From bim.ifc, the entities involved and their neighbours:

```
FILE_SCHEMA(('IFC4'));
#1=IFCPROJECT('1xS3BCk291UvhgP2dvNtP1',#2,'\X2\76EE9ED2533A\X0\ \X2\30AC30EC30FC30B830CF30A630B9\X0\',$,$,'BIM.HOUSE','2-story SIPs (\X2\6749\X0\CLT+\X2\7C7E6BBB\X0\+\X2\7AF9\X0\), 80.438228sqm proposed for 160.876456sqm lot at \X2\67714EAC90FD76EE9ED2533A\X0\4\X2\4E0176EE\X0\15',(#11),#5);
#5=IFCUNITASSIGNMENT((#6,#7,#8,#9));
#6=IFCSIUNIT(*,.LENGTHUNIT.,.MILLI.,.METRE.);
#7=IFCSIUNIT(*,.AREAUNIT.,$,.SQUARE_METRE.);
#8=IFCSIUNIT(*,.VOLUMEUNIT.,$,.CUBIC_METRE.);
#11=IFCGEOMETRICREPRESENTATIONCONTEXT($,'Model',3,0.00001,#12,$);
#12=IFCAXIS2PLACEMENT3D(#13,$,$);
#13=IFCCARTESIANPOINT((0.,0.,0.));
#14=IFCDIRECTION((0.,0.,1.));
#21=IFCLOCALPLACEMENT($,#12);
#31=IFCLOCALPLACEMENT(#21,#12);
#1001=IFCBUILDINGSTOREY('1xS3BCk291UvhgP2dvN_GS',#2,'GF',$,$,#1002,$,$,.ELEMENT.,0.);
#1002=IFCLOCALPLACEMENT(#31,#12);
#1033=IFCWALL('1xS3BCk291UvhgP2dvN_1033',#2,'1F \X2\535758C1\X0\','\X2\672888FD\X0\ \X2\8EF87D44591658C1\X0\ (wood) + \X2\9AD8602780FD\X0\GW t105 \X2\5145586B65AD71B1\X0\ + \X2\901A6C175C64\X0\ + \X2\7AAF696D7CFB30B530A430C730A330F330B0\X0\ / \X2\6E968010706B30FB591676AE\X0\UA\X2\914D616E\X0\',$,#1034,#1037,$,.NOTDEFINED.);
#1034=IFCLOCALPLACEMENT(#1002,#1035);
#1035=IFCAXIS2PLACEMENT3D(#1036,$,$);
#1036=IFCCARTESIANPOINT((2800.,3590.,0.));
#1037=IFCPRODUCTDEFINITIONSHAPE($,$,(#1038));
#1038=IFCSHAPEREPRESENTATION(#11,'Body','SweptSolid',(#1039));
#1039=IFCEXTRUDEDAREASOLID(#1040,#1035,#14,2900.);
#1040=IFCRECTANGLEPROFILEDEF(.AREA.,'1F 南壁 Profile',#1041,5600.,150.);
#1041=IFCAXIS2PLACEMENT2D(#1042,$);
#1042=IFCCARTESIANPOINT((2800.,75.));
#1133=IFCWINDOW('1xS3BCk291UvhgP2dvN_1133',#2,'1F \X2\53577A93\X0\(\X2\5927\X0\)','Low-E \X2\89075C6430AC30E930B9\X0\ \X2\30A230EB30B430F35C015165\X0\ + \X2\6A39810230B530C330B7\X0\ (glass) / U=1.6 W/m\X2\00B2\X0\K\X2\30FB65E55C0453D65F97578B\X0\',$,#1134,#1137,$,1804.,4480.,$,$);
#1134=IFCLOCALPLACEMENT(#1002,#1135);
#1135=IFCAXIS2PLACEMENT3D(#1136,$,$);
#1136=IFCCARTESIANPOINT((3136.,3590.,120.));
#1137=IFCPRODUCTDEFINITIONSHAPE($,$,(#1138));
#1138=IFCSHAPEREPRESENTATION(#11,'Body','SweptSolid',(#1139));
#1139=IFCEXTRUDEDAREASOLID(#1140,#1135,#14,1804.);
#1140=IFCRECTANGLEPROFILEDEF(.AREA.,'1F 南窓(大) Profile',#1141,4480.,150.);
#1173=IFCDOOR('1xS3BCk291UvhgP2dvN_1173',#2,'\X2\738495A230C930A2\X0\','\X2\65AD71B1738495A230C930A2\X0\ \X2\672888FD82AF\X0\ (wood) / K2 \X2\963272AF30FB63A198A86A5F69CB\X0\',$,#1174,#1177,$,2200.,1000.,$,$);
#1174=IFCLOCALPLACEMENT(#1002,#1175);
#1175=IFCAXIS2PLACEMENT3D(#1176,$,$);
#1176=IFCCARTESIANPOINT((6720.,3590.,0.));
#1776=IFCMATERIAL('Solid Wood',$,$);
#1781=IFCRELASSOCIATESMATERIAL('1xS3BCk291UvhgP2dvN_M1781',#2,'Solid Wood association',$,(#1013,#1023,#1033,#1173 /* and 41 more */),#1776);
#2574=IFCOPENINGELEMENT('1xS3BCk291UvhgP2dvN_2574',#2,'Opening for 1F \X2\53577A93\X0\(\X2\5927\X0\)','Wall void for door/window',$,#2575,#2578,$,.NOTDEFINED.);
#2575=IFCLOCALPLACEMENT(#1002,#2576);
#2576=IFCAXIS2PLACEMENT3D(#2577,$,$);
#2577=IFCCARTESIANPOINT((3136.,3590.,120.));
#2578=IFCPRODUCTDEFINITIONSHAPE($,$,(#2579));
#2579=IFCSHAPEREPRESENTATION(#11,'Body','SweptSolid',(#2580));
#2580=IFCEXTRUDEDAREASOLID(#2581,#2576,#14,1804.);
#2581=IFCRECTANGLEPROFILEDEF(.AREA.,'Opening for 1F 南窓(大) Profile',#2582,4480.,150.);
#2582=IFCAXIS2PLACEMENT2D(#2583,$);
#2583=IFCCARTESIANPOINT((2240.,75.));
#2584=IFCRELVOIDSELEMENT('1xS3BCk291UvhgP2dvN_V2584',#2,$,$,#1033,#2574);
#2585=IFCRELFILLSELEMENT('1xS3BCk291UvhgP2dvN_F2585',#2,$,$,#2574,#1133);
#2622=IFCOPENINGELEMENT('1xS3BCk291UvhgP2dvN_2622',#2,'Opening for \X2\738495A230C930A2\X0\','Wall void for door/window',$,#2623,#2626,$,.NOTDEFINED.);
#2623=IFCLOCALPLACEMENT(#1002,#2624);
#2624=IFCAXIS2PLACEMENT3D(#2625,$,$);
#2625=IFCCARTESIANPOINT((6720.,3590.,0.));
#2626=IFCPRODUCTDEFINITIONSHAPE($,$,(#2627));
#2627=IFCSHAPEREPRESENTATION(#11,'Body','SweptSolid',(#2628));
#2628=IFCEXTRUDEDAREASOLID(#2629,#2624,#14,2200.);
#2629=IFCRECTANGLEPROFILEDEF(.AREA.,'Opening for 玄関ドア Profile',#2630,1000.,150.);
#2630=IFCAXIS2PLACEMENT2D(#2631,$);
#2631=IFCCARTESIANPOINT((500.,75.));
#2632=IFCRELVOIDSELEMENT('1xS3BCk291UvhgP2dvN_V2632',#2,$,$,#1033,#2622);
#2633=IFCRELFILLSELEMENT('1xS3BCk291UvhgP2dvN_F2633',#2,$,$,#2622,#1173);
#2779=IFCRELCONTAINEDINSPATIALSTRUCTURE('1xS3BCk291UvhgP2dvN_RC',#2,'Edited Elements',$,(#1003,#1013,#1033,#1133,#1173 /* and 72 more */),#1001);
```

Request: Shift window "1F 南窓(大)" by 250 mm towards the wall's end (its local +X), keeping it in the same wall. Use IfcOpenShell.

```python
import ifcopenshell
import ifcopenshell.api.geometry
import ifcopenshell.util.placement

model = ifcopenshell.open("bim.ifc")

window = model.by_guid("1xS3BCk291UvhgP2dvN_1133")
opening = window.FillsVoids[0].RelatingOpeningElement
wall = opening.VoidsElements[0].RelatingBuildingElement

wall_matrix = ifcopenshell.util.placement.get_local_placement(wall.ObjectPlacement)
shift = wall_matrix[:3, 0] * 250.0
before = ifcopenshell.util.placement.get_local_placement(window.ObjectPlacement)[:3, 3].copy()

# The window is not placed relative to its opening, so move both.
for product in (opening, window):
    matrix = ifcopenshell.util.placement.get_local_placement(product.ObjectPlacement)
    matrix[:3, 3] += shift
    ifcopenshell.api.geometry.edit_object_placement(model, product=product, matrix=matrix, is_si=False)

after = ifcopenshell.util.placement.get_local_placement(window.ObjectPlacement)[:3, 3]
print("window moved by", (after - before).round(3) + 0.0)

model.write("bim-out.ifc")
```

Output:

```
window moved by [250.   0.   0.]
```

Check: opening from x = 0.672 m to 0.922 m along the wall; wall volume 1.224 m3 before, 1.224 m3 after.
